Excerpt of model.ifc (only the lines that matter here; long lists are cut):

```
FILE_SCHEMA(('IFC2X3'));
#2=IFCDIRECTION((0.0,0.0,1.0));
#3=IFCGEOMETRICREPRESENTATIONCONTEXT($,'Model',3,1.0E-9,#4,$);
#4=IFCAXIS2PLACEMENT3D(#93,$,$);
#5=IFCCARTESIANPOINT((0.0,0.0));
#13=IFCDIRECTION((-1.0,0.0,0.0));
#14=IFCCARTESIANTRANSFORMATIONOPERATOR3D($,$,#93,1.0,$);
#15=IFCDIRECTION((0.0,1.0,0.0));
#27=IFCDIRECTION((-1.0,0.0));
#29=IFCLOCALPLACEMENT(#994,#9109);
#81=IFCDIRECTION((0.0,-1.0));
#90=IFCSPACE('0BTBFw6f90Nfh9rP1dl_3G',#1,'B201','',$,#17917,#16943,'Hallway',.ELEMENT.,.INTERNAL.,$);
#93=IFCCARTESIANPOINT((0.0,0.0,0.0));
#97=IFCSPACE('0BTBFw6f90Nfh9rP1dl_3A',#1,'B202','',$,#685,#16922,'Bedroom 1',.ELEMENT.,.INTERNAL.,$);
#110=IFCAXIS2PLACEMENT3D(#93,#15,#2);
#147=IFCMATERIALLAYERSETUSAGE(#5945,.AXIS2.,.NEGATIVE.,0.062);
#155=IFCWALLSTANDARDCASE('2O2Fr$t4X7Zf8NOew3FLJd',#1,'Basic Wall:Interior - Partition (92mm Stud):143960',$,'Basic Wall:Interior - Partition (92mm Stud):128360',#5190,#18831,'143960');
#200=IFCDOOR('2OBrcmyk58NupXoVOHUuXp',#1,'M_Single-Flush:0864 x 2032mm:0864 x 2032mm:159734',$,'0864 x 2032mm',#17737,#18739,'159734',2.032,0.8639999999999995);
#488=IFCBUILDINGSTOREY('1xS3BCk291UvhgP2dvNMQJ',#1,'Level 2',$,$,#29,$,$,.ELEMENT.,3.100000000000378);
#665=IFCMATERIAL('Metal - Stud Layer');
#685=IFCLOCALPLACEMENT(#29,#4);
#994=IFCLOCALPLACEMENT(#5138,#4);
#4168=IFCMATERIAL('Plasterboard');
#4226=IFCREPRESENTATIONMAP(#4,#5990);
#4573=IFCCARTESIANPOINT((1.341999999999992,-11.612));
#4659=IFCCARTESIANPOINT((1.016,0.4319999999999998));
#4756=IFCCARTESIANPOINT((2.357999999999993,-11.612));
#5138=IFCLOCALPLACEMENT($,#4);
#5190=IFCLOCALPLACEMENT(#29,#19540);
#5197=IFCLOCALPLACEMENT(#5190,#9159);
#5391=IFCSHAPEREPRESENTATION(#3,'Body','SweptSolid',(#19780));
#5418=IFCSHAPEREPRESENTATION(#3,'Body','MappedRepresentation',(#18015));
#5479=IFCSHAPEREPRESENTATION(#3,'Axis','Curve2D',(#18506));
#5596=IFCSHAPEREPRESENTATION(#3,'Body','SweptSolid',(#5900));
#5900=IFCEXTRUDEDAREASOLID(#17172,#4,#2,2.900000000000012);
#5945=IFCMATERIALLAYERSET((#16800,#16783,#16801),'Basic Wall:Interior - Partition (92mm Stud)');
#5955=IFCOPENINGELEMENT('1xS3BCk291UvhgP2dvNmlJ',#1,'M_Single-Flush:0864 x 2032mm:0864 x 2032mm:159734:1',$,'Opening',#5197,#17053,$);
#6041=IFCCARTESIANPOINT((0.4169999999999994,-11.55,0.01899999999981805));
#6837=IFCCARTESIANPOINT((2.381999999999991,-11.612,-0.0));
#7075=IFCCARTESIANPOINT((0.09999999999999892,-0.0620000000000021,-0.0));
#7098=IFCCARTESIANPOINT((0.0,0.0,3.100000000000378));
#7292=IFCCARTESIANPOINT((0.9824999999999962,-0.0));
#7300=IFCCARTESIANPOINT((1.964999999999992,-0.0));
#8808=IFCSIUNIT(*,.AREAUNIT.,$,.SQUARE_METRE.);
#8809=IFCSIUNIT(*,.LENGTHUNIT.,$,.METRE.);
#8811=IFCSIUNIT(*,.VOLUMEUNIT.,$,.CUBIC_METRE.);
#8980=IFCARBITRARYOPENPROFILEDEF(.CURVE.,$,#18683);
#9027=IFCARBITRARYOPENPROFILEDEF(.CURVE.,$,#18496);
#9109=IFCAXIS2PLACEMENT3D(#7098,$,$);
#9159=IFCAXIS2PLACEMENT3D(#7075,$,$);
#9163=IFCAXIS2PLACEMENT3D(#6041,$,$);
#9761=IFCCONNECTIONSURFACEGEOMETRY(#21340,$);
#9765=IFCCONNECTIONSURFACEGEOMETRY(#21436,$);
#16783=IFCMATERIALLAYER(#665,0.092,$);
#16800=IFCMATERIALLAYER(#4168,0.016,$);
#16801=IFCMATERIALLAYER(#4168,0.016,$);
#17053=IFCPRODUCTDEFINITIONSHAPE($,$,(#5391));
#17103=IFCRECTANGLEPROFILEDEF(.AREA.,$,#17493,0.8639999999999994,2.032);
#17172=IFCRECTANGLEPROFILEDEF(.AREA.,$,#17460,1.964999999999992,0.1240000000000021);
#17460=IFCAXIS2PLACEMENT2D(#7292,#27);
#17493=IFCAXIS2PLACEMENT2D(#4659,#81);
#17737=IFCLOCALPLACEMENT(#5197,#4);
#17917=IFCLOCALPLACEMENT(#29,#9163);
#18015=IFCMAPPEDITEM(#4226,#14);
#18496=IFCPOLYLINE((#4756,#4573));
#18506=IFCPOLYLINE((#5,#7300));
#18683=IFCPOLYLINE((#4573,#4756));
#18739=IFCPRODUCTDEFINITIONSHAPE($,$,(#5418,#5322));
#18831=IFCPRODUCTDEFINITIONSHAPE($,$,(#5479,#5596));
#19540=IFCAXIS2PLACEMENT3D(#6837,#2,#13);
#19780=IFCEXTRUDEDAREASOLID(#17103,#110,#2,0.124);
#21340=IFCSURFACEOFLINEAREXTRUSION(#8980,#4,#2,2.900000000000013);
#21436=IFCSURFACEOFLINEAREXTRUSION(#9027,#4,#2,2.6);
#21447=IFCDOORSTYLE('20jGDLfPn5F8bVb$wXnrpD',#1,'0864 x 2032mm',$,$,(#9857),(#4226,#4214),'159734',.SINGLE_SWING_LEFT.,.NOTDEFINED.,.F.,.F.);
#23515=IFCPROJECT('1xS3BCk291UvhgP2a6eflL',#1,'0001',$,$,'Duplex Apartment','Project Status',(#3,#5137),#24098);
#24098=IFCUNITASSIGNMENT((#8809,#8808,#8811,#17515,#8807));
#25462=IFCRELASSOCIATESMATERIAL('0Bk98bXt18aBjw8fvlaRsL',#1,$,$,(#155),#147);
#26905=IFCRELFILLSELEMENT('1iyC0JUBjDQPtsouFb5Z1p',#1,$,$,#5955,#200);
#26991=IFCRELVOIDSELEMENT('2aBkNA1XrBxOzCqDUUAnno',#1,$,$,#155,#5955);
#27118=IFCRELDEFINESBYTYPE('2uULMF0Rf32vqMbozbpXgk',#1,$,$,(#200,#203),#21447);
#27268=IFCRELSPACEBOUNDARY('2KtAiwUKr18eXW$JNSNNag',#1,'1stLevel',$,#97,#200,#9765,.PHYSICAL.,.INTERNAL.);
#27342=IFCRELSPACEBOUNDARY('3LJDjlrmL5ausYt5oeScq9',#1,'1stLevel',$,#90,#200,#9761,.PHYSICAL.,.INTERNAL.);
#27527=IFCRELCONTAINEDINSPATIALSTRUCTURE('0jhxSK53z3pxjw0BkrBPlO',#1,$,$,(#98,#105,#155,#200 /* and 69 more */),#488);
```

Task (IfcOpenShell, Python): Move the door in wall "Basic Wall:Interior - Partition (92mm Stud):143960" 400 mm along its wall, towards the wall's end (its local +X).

```python
import numpy as np
import ifcopenshell
import ifcopenshell.api.geometry
import ifcopenshell.util.placement
import ifcopenshell.util.unit

model = ifcopenshell.open("model.ifc")
unit_scale = ifcopenshell.util.unit.calculate_unit_scale(model)

door = model.by_guid("2OBrcmyk58NupXoVOHUuXp")
opening = door.FillsVoids[0].RelatingOpeningElement
wall = opening.VoidsElements[0].RelatingBuildingElement

wall_matrix = ifcopenshell.util.placement.get_local_placement(wall.ObjectPlacement)
shift = wall_matrix[:3, 0] * 0.4 / unit_scale
before = ifcopenshell.util.placement.get_local_placement(door.ObjectPlacement)[:3, 3].copy()

# The door is placed relative to its opening, so it follows when the opening moves.
matrix = ifcopenshell.util.placement.get_local_placement(opening.ObjectPlacement)
matrix[:3, 3] += shift
ifcopenshell.api.geometry.edit_object_placement(
    model, product=opening, matrix=matrix, is_si=False, should_transform_children=True
)

# Space boundary surfaces are stored in each space's coordinates; move them too.
for rel in door.ProvidesBoundaries:
    if not rel.ConnectionGeometry:
        continue
    surface = rel.ConnectionGeometry.SurfaceOnRelatingElement
    space_matrix = ifcopenshell.util.placement.get_local_placement(rel.RelatingSpace.ObjectPlacement)
    point = np.array(surface.Position.Location.Coordinates) + space_matrix[:3, :3].T @ shift
    surface.Position = model.createIfcAxis2Placement3D(
        model.createIfcCartesianPoint(point.tolist()), surface.Position.Axis, surface.Position.RefDirection
    )

after = ifcopenshell.util.placement.get_local_placement(door.ObjectPlacement)[:3, 3]
print("door moved by", (after - before).round(3) + 0.0)

model.write("model_updated.ifc")
```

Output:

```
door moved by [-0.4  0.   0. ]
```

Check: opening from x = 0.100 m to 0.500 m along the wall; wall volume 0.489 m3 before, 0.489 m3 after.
